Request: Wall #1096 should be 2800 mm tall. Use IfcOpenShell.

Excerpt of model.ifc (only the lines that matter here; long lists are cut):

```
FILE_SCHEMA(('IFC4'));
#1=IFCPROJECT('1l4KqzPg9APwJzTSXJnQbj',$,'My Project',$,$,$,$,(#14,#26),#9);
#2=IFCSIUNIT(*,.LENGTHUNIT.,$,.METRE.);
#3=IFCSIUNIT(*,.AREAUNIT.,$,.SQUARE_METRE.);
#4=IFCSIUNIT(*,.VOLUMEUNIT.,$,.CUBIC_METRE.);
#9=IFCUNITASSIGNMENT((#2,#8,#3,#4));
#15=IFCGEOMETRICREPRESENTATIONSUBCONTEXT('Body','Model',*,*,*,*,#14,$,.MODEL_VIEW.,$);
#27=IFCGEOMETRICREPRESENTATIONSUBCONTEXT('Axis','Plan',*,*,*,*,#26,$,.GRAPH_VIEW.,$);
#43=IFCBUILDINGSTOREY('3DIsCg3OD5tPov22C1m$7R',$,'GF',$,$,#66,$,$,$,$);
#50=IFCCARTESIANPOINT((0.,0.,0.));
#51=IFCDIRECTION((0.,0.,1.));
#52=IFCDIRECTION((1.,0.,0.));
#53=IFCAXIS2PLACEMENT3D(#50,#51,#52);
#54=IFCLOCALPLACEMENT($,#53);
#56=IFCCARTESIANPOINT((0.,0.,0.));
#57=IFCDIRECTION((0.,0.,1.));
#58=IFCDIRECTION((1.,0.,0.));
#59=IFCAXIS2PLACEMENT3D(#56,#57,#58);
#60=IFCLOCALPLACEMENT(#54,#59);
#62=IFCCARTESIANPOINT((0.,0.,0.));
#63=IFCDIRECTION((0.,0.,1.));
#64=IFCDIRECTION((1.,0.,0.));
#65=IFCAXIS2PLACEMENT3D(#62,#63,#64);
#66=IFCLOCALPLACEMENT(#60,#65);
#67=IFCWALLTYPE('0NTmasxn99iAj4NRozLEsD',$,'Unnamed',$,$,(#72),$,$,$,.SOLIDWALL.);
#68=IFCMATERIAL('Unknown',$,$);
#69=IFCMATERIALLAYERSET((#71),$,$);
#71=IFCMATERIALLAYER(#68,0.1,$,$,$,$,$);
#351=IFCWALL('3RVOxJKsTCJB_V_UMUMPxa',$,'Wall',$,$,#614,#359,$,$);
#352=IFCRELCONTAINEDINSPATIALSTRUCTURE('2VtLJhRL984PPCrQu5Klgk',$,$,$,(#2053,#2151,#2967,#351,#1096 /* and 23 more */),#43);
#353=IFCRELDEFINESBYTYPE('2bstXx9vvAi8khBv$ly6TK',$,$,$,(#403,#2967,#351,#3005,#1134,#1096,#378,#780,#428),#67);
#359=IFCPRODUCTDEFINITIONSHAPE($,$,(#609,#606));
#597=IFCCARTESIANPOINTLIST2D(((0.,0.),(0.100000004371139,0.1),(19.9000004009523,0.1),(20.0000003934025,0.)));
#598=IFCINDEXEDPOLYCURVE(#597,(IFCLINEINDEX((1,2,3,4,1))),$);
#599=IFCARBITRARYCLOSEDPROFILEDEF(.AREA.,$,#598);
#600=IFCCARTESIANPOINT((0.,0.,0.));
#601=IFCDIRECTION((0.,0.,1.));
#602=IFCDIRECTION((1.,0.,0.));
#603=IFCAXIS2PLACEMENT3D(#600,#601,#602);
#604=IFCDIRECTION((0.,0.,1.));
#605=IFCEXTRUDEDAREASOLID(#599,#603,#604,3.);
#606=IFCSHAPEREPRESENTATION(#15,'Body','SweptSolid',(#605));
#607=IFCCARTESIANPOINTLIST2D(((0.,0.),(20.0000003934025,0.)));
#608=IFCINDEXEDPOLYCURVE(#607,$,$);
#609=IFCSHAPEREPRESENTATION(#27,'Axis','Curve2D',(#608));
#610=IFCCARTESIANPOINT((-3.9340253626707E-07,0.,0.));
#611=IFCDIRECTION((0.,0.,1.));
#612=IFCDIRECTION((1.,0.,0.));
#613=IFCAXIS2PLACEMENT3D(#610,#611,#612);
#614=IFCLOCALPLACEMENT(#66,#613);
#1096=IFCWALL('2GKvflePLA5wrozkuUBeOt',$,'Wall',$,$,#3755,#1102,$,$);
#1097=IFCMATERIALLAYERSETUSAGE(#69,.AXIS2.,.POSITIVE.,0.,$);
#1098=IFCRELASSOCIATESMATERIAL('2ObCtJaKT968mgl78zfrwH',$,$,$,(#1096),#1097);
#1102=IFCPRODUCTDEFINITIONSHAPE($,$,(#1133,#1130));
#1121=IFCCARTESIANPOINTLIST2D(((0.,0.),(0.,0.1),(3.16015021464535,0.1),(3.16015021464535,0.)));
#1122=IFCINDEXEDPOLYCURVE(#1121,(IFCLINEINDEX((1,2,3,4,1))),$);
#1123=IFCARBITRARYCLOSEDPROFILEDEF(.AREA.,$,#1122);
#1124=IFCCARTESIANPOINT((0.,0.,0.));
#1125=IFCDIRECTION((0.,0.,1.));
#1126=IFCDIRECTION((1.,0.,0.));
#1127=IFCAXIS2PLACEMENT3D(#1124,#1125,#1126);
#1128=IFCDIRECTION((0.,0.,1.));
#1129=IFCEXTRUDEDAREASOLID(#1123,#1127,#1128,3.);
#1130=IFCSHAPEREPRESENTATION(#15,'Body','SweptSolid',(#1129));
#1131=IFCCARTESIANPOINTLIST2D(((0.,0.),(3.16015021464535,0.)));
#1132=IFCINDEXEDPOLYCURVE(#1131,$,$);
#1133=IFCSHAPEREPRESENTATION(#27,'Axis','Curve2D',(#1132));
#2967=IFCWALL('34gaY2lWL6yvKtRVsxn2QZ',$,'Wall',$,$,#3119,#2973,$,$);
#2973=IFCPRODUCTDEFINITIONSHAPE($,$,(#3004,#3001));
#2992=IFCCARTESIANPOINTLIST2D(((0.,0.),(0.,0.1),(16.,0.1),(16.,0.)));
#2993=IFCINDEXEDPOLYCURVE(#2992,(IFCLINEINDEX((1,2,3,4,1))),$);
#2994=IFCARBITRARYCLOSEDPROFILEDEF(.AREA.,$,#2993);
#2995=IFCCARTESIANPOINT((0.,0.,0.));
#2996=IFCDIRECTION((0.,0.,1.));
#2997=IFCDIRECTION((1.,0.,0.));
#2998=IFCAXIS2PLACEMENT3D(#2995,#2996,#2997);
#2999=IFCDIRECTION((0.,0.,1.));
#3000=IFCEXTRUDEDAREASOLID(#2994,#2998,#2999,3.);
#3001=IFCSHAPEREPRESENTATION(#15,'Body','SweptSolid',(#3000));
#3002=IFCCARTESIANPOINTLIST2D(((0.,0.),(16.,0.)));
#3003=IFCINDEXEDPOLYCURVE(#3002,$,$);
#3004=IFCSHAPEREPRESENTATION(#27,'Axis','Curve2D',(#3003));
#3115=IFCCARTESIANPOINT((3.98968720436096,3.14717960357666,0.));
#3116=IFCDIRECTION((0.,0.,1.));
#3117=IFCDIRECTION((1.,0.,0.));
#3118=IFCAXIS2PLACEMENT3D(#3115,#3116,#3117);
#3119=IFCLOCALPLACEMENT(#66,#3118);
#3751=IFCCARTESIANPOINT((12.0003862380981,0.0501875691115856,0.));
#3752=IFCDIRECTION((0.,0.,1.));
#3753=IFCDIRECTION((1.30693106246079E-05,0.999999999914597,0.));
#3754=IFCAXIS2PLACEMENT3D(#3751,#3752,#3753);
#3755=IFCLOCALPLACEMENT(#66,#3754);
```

```python
import ifcopenshell
import ifcopenshell.geom
import ifcopenshell.util.representation
import ifcopenshell.util.shape

model = ifcopenshell.open("model.ifc")
settings = ifcopenshell.geom.settings()


def volume(element):
    """Net volume in cubic metres, openings subtracted."""
    shape = ifcopenshell.geom.create_shape(settings, element)
    return ifcopenshell.util.shape.get_volume(shape.geometry)


wall = model.by_id(1096)
before = volume(wall)

body = ifcopenshell.util.representation.get_representation(wall, "Model", "Body")
solid = body.Items[0]
old_height = solid.Depth
solid.Depth = 2.8
after = volume(wall)

print(f"height {old_height:g} -> {solid.Depth:g}, volume {before:.3f} -> {after:.3f} m3")

model.write("model-out.ifc")
```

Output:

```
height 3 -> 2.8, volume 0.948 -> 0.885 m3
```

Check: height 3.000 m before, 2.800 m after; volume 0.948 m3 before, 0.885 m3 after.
